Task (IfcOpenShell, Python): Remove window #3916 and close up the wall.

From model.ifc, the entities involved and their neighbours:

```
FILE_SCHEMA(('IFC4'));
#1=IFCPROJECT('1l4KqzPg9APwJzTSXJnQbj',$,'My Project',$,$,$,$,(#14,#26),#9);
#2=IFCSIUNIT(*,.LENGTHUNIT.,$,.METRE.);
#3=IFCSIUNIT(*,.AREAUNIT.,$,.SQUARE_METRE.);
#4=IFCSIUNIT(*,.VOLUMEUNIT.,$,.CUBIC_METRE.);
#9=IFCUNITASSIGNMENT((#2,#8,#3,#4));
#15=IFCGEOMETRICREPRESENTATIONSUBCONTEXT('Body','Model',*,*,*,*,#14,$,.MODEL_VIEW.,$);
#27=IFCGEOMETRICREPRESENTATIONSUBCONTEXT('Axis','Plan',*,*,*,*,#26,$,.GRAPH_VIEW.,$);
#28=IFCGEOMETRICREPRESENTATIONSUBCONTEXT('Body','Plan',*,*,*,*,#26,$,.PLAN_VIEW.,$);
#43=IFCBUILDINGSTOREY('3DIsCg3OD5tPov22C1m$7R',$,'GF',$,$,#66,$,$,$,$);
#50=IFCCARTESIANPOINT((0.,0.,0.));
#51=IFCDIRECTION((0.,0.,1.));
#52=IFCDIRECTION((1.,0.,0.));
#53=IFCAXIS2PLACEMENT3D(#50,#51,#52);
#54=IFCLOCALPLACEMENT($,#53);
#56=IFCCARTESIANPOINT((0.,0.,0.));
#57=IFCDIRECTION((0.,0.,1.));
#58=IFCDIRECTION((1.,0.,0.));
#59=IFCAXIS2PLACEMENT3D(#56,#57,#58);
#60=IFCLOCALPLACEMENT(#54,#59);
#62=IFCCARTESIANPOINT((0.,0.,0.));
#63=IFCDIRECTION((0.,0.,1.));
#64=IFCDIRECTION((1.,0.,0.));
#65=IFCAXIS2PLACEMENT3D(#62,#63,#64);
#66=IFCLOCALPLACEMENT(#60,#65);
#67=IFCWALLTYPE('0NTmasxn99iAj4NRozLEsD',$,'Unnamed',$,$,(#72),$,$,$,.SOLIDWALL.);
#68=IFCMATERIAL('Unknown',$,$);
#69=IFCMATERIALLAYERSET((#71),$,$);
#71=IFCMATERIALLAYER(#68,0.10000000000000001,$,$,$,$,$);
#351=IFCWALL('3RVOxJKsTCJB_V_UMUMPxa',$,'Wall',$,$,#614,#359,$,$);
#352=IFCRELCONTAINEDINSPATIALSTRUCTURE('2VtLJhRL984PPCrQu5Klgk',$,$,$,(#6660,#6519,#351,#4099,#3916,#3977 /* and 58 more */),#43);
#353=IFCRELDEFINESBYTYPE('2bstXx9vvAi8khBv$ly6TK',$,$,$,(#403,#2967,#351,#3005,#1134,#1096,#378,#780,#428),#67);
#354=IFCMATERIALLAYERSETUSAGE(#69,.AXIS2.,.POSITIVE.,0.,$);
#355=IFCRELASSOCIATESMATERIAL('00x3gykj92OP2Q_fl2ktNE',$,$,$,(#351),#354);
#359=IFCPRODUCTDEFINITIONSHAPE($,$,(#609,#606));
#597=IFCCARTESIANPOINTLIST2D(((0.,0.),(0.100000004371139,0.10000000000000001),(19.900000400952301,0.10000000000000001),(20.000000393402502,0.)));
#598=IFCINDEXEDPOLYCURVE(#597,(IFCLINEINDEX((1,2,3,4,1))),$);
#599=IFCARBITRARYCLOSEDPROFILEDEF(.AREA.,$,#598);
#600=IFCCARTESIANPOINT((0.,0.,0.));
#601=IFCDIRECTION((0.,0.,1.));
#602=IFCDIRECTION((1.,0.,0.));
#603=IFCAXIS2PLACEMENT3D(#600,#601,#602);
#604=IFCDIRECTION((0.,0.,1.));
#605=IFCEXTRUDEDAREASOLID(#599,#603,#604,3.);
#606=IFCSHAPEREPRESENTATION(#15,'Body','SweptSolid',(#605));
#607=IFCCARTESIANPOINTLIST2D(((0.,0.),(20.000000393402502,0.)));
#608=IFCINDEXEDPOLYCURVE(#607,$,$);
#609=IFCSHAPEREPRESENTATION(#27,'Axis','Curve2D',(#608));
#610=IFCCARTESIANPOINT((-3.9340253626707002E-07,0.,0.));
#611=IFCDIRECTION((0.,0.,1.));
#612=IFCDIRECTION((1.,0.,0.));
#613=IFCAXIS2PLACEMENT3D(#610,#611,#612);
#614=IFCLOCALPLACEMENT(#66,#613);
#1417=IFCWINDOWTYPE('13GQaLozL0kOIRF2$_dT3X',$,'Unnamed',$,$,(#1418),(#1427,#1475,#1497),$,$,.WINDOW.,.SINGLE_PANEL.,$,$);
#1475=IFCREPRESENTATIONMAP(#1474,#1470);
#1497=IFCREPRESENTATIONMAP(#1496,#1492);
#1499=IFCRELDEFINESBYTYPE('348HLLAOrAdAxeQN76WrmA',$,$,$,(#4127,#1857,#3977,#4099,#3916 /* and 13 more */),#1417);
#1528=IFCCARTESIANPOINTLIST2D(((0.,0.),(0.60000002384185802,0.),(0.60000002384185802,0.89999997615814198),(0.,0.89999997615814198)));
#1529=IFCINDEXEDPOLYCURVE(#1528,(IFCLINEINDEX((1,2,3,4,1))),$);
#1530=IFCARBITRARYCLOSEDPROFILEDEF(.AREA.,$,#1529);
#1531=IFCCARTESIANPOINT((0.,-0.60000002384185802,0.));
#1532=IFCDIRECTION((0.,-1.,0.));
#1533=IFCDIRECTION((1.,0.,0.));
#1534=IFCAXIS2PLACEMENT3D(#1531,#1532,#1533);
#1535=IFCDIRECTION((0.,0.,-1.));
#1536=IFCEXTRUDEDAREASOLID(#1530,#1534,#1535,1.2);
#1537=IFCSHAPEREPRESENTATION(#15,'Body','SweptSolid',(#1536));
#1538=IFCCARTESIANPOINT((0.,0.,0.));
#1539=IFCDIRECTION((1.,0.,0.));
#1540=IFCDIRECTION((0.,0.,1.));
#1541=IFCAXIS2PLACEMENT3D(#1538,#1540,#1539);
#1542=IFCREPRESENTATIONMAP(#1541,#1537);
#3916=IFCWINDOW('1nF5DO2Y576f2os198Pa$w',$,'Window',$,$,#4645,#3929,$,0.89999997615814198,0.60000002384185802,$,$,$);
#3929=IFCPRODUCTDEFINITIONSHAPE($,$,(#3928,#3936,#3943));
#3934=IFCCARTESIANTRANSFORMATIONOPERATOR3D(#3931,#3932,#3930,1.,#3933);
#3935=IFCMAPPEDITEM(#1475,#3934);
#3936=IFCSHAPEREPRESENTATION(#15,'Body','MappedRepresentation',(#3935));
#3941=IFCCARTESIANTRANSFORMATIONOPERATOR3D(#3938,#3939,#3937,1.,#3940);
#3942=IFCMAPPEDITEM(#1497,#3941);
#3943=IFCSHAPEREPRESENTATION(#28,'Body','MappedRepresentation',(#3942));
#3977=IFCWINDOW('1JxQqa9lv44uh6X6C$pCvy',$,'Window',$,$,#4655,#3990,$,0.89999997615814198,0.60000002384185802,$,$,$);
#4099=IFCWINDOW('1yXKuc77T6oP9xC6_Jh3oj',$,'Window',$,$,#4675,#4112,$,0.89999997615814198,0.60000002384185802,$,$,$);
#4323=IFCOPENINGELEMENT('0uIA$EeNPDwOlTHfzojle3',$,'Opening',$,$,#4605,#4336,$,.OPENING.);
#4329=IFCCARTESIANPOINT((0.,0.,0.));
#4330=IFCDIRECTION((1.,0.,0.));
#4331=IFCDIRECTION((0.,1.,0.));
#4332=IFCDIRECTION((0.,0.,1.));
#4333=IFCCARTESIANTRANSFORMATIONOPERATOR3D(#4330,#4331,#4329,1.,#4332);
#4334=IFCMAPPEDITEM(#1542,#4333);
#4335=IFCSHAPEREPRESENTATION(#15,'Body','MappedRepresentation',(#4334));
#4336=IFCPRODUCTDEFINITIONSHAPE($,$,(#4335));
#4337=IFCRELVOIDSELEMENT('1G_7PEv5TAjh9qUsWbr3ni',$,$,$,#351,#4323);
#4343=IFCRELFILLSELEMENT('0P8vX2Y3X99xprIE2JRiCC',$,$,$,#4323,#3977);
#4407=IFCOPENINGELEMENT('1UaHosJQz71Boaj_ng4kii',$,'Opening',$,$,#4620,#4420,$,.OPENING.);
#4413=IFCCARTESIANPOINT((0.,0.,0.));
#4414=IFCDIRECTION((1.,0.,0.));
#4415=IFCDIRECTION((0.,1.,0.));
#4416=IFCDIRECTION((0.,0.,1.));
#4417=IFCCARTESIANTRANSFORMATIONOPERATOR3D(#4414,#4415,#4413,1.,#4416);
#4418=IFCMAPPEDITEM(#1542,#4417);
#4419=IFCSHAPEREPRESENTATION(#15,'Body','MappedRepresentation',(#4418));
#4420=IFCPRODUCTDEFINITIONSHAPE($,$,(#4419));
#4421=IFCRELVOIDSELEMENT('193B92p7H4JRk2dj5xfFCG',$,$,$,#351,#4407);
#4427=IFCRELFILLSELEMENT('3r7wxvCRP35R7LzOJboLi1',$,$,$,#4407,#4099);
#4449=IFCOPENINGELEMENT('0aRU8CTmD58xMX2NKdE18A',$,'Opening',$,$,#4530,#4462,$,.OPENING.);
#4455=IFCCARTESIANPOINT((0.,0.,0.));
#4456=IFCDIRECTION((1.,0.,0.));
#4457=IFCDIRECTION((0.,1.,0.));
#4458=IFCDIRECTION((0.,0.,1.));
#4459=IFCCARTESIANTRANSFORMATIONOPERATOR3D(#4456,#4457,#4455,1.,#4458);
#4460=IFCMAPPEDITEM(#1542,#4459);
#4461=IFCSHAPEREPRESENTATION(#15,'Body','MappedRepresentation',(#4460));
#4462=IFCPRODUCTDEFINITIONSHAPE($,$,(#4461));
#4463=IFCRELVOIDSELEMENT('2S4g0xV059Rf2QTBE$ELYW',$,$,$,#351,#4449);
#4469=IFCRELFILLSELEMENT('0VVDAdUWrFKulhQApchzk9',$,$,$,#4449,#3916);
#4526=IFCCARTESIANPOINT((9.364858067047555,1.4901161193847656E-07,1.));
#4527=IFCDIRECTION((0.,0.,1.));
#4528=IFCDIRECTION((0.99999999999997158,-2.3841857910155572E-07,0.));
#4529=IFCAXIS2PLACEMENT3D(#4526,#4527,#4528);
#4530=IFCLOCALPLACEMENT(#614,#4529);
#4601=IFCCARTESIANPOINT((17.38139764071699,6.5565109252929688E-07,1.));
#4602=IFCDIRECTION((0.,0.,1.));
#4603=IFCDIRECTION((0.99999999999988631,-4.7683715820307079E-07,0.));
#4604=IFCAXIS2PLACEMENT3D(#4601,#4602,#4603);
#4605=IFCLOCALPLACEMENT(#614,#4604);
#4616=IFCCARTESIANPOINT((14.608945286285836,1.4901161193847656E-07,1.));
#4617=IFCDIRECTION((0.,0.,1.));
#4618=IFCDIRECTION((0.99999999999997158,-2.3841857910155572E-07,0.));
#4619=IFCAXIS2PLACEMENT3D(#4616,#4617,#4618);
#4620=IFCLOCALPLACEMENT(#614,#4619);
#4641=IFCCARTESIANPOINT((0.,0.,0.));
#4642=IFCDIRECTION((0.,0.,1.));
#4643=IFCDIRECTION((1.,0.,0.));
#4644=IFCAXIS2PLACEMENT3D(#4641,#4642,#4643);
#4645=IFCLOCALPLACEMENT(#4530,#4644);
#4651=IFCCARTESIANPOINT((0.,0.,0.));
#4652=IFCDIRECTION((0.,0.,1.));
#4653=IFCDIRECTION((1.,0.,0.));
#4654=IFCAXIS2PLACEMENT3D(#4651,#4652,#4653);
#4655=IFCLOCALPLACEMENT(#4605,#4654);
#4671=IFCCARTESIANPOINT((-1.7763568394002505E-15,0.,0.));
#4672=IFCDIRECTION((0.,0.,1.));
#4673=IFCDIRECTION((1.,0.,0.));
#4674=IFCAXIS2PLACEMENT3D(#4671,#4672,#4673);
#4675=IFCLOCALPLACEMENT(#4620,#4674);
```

```python
import ifcopenshell
import ifcopenshell.api.feature
import ifcopenshell.api.root
import ifcopenshell.geom
import ifcopenshell.util.shape

model = ifcopenshell.open("model.ifc")
settings = ifcopenshell.geom.settings()


def volume(element):
    """Net volume in cubic metres, openings subtracted."""
    shape = ifcopenshell.geom.create_shape(settings, element)
    return ifcopenshell.util.shape.get_volume(shape.geometry)


window = model.by_guid("1nF5DO2Y576f2os198Pa$w")
opening = window.FillsVoids[0].RelatingOpeningElement
wall = opening.VoidsElements[0].RelatingBuildingElement
before = volume(wall)

ifcopenshell.api.root.remove_product(model, product=window)
ifcopenshell.api.feature.remove_feature(model, feature=opening)

after = volume(wall)

print(f"wall volume {before:.3f} -> {after:.3f} m3")

model.write("model_updated.ifc")
```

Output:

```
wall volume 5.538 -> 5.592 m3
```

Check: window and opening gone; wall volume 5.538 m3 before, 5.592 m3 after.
